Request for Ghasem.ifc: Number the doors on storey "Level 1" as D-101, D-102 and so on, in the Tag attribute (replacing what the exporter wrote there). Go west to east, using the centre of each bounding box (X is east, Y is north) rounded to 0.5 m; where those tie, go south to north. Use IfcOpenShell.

First a look at what the model holds.

```python
import ifcopenshell
import ifcopenshell.util.element
import ifcopenshell.util.placement

model = ifcopenshell.open("Ghasem.ifc")
print(model.schema)
storey = next(s for s in model.by_type("IfcBuildingStorey") if s.Name == "Level 1")
doors = [e for e in ifcopenshell.util.element.get_decomposition(storey) if e.is_a("IfcDoor")]
for e in sorted(doors, key=lambda e: e.id()):
    origin = ifcopenshell.util.placement.get_local_placement(e.ObjectPlacement)[:3, 3]
    print(e.id(), e.Tag, e.Name, origin.round(2) + 0.0, sep=" | ")
```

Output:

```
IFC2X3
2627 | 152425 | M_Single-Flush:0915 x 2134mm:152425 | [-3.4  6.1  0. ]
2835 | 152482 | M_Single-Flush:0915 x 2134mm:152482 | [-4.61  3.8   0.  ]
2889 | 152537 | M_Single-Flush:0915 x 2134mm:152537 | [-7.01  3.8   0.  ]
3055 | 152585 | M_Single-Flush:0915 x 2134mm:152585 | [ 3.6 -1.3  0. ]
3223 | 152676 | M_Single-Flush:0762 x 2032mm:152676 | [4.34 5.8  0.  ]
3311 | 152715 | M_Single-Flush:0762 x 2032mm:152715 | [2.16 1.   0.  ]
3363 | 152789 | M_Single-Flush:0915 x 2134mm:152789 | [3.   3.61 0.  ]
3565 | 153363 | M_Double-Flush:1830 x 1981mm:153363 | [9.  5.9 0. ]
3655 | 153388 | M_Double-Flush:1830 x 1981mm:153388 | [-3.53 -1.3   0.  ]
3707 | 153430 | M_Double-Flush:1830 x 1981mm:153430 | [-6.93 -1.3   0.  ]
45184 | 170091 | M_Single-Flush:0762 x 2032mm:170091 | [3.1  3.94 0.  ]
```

```python
import ifcopenshell
import ifcopenshell.geom
import ifcopenshell.util.element
import ifcopenshell.util.shape

model = ifcopenshell.open("Ghasem.ifc")
settings = ifcopenshell.geom.settings()
settings.set("use-world-coords", True)


def centre(element):
    shape = ifcopenshell.geom.create_shape(settings, element)
    return ifcopenshell.util.shape.get_bbox_centroid(shape.geometry)


storey = next(s for s in model.by_type("IfcBuildingStorey") if s.Name == "Level 1")
doors = [e for e in ifcopenshell.util.element.get_decomposition(storey) if e.is_a("IfcDoor")]

# Insertion points can sit at a corner or the storey origin, so sort by the geometry (in metres).
centres = {e: centre(e) for e in doors}
doors.sort(key=lambda e: (round(centres[e][0] / 0.5), centres[e][1]))

for i, e in enumerate(doors, start=1):
    number = f"D-1{i:02d}"
    e.Tag = number
    print(e.id(), number)

model.write("Ghasem_updated.ifc")
```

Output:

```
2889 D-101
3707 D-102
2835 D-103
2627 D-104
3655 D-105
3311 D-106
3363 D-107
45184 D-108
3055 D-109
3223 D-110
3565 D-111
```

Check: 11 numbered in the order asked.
